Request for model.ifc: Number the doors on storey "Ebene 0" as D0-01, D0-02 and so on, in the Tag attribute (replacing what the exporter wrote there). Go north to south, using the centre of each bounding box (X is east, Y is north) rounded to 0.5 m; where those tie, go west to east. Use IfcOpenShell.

First a look at what the model holds.

```python
import ifcopenshell
import ifcopenshell.util.element
import ifcopenshell.util.placement

model = ifcopenshell.open("model.ifc")
print(model.schema)
storey = next(s for s in model.by_type("IfcBuildingStorey") if s.Name == "Ebene 0")
doors = [e for e in ifcopenshell.util.element.get_decomposition(storey) if e.is_a("IfcDoor")]
for e in sorted(doors, key=lambda e: e.id()):
    origin = ifcopenshell.util.placement.get_local_placement(e.ObjectPlacement)[:3, 3]
    print(e.id(), e.Tag, e.Name, origin.round(2) + 0.0, sep=" | ")
```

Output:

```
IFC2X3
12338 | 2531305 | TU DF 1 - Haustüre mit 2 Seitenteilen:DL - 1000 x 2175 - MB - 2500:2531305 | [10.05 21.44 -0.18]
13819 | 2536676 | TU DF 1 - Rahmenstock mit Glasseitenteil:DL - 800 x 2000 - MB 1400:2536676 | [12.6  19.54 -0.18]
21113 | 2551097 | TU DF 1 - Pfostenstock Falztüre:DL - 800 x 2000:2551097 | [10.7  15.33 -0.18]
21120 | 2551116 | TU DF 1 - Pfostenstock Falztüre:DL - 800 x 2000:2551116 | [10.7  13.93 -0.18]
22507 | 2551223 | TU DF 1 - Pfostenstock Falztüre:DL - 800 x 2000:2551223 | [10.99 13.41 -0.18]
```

```python
import ifcopenshell
import ifcopenshell.geom
import ifcopenshell.util.element
import ifcopenshell.util.shape

model = ifcopenshell.open("model.ifc")
settings = ifcopenshell.geom.settings()
settings.set("use-world-coords", True)


def centre(element):
    shape = ifcopenshell.geom.create_shape(settings, element)
    return ifcopenshell.util.shape.get_bbox_centroid(shape.geometry)


storey = next(s for s in model.by_type("IfcBuildingStorey") if s.Name == "Ebene 0")
doors = [e for e in ifcopenshell.util.element.get_decomposition(storey) if e.is_a("IfcDoor")]

# Insertion points can sit at a corner or the storey origin, so sort by the geometry (in metres).
centres = {e: centre(e) for e in doors}
doors.sort(key=lambda e: (-round(centres[e][1] / 0.5), centres[e][0]))

for i, e in enumerate(doors, start=1):
    number = f"D0-{i:02d}"
    e.Tag = number
    print(e.id(), number)

model.write("model-out.ifc")
```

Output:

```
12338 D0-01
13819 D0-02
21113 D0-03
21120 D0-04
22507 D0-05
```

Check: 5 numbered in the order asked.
